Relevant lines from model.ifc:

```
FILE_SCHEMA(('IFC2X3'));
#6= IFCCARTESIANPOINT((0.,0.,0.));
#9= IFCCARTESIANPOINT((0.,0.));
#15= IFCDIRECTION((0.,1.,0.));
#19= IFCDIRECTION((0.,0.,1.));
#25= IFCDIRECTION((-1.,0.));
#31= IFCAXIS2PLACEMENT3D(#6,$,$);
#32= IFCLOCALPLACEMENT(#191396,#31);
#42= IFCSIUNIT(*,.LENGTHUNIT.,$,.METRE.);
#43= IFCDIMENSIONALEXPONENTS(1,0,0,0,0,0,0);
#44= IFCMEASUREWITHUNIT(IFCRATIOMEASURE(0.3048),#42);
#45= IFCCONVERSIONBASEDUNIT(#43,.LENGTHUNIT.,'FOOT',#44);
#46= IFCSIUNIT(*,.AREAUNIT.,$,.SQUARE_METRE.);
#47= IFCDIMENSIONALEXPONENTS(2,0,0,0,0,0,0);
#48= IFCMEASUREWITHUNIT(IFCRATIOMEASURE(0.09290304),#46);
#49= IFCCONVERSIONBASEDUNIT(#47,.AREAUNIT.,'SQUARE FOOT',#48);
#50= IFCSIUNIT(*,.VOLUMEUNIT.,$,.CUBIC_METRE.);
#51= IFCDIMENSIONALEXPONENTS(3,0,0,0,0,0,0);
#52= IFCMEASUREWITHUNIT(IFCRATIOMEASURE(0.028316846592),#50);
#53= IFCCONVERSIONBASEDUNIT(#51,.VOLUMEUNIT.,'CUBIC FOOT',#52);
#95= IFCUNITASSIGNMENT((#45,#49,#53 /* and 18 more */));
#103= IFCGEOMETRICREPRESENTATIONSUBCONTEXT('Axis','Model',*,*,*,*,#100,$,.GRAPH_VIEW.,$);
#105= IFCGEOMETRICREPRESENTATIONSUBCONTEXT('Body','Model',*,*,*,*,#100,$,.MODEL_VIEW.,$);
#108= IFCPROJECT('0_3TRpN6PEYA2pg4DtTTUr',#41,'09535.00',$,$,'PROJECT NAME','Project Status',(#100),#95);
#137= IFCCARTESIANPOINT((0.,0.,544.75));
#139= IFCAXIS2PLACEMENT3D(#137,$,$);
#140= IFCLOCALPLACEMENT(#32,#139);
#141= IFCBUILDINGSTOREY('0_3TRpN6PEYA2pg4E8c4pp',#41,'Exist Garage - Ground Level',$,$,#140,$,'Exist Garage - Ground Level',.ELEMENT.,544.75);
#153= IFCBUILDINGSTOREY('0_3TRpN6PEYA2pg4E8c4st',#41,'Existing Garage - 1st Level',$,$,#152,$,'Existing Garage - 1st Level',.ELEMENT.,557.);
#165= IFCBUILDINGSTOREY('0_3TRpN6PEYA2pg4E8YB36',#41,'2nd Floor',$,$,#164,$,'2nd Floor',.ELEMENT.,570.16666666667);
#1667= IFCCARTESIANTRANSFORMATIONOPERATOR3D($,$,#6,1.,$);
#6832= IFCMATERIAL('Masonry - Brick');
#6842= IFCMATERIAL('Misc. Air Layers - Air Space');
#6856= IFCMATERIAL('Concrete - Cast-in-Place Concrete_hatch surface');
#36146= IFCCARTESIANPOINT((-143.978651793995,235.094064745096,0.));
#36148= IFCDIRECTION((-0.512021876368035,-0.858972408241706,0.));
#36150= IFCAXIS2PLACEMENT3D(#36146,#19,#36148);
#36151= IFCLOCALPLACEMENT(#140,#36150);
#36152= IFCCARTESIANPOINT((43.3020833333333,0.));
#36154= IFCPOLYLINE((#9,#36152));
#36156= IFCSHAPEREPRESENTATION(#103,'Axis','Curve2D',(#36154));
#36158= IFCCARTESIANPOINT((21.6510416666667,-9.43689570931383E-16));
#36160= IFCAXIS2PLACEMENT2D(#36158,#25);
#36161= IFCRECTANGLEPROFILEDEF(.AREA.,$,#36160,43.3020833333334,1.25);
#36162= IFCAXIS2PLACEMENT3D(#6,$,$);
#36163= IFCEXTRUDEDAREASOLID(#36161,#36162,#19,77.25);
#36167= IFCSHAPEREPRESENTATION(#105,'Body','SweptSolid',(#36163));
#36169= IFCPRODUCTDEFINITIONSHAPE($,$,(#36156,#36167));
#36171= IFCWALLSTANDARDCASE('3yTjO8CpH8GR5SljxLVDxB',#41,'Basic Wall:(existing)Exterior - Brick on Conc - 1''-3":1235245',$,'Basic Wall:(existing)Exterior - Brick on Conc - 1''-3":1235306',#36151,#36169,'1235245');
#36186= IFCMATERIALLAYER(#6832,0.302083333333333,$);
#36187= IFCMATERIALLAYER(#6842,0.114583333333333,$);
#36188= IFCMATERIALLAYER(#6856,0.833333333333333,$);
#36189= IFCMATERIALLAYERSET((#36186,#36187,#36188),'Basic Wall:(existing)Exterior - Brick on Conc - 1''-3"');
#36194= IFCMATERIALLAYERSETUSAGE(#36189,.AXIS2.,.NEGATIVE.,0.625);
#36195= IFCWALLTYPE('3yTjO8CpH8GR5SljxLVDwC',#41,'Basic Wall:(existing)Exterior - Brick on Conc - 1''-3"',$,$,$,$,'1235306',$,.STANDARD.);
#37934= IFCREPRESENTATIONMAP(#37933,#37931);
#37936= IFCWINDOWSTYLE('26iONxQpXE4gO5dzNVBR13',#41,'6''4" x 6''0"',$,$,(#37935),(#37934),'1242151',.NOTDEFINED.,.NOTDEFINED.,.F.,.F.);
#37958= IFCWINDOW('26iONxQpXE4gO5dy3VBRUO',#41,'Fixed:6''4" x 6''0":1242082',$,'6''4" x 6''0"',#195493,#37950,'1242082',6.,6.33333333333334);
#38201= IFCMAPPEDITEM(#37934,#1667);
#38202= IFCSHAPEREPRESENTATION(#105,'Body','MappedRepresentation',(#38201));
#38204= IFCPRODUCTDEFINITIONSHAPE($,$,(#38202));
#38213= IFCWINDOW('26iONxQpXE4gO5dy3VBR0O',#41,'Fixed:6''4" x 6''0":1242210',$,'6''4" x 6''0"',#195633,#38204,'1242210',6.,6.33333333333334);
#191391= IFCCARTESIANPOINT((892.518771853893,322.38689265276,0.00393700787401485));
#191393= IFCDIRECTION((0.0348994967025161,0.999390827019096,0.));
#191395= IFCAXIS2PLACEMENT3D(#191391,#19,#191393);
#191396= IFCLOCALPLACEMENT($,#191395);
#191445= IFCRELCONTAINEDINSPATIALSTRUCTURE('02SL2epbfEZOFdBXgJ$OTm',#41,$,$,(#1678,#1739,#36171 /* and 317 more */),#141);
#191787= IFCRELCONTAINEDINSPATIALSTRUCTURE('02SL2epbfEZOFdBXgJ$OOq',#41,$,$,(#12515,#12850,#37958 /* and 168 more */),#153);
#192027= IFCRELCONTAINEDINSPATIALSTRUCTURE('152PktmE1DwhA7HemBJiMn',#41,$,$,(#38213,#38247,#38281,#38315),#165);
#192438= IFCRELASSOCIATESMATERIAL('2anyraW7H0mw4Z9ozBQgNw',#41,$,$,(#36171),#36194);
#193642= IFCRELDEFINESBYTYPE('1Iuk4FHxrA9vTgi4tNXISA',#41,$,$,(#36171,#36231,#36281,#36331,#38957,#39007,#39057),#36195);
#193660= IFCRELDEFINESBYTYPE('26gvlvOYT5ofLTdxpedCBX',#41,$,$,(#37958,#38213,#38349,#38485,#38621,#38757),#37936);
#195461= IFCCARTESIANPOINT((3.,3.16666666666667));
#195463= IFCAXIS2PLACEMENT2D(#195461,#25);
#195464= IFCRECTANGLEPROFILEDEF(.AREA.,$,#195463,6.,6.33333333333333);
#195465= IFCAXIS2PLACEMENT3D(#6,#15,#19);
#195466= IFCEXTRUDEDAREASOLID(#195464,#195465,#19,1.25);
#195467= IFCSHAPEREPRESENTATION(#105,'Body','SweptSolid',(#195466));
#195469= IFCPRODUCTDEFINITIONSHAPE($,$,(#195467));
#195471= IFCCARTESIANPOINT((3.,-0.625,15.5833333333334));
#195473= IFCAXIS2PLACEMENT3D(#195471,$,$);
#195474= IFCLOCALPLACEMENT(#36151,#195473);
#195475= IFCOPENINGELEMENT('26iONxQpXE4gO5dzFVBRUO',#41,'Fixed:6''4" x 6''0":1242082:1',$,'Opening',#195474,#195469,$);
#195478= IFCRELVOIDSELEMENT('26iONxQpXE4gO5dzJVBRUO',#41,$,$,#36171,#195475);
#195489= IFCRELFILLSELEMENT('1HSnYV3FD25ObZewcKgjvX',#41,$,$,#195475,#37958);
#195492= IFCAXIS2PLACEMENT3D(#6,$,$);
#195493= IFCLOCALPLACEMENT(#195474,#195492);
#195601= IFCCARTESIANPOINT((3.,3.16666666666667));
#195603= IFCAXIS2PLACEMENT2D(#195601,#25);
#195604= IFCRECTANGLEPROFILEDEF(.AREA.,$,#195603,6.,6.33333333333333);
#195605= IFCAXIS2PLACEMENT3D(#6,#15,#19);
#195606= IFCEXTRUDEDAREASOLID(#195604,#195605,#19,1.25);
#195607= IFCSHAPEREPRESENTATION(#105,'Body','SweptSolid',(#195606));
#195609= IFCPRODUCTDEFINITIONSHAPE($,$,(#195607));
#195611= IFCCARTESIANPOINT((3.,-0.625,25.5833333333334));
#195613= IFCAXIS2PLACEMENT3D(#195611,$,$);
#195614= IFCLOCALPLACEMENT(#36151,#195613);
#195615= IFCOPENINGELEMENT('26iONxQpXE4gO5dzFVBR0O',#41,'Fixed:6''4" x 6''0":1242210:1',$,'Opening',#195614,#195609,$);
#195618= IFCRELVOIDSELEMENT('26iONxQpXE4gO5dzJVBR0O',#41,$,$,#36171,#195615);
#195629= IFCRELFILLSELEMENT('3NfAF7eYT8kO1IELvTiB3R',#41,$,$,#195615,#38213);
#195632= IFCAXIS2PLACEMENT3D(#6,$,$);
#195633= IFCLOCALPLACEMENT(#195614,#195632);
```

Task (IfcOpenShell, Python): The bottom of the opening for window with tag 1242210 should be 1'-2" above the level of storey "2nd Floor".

```python
import numpy as np
import ifcopenshell
import ifcopenshell.api.geometry
import ifcopenshell.geom
import ifcopenshell.util.element
import ifcopenshell.util.placement
import ifcopenshell.util.shape
import ifcopenshell.util.unit

model = ifcopenshell.open("model.ifc")
unit_scale = ifcopenshell.util.unit.calculate_unit_scale(model)

window = model.by_guid("26iONxQpXE4gO5dy3VBR0O")
opening = window.FillsVoids[0].RelatingOpeningElement
storey = ifcopenshell.util.element.get_container(window, ifc_class="IfcBuildingStorey")
level = ifcopenshell.util.placement.get_local_placement(storey.ObjectPlacement)[2, 3]

# The opening's origin need not be at the sill, so measure its lowest point.
shape = ifcopenshell.geom.create_shape(ifcopenshell.geom.settings(), opening)
bottom = ifcopenshell.util.shape.get_shape_bottom_elevation(shape, shape.geometry) / unit_scale
dz = level + 14 * 0.0254 / unit_scale - bottom

shift = np.array([0.0, 0.0, dz])
# The window is placed relative to its opening, so it follows when the opening moves.
matrix = ifcopenshell.util.placement.get_local_placement(opening.ObjectPlacement)
matrix[:3, 3] += shift
ifcopenshell.api.geometry.edit_object_placement(
    model, product=opening, matrix=matrix, is_si=False, should_transform_children=True
)

print(f"moved by {dz * unit_scale:+.3f} m")

model.write("model_rev.ifc")
```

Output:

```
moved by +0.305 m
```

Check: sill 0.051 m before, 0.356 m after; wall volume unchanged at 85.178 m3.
